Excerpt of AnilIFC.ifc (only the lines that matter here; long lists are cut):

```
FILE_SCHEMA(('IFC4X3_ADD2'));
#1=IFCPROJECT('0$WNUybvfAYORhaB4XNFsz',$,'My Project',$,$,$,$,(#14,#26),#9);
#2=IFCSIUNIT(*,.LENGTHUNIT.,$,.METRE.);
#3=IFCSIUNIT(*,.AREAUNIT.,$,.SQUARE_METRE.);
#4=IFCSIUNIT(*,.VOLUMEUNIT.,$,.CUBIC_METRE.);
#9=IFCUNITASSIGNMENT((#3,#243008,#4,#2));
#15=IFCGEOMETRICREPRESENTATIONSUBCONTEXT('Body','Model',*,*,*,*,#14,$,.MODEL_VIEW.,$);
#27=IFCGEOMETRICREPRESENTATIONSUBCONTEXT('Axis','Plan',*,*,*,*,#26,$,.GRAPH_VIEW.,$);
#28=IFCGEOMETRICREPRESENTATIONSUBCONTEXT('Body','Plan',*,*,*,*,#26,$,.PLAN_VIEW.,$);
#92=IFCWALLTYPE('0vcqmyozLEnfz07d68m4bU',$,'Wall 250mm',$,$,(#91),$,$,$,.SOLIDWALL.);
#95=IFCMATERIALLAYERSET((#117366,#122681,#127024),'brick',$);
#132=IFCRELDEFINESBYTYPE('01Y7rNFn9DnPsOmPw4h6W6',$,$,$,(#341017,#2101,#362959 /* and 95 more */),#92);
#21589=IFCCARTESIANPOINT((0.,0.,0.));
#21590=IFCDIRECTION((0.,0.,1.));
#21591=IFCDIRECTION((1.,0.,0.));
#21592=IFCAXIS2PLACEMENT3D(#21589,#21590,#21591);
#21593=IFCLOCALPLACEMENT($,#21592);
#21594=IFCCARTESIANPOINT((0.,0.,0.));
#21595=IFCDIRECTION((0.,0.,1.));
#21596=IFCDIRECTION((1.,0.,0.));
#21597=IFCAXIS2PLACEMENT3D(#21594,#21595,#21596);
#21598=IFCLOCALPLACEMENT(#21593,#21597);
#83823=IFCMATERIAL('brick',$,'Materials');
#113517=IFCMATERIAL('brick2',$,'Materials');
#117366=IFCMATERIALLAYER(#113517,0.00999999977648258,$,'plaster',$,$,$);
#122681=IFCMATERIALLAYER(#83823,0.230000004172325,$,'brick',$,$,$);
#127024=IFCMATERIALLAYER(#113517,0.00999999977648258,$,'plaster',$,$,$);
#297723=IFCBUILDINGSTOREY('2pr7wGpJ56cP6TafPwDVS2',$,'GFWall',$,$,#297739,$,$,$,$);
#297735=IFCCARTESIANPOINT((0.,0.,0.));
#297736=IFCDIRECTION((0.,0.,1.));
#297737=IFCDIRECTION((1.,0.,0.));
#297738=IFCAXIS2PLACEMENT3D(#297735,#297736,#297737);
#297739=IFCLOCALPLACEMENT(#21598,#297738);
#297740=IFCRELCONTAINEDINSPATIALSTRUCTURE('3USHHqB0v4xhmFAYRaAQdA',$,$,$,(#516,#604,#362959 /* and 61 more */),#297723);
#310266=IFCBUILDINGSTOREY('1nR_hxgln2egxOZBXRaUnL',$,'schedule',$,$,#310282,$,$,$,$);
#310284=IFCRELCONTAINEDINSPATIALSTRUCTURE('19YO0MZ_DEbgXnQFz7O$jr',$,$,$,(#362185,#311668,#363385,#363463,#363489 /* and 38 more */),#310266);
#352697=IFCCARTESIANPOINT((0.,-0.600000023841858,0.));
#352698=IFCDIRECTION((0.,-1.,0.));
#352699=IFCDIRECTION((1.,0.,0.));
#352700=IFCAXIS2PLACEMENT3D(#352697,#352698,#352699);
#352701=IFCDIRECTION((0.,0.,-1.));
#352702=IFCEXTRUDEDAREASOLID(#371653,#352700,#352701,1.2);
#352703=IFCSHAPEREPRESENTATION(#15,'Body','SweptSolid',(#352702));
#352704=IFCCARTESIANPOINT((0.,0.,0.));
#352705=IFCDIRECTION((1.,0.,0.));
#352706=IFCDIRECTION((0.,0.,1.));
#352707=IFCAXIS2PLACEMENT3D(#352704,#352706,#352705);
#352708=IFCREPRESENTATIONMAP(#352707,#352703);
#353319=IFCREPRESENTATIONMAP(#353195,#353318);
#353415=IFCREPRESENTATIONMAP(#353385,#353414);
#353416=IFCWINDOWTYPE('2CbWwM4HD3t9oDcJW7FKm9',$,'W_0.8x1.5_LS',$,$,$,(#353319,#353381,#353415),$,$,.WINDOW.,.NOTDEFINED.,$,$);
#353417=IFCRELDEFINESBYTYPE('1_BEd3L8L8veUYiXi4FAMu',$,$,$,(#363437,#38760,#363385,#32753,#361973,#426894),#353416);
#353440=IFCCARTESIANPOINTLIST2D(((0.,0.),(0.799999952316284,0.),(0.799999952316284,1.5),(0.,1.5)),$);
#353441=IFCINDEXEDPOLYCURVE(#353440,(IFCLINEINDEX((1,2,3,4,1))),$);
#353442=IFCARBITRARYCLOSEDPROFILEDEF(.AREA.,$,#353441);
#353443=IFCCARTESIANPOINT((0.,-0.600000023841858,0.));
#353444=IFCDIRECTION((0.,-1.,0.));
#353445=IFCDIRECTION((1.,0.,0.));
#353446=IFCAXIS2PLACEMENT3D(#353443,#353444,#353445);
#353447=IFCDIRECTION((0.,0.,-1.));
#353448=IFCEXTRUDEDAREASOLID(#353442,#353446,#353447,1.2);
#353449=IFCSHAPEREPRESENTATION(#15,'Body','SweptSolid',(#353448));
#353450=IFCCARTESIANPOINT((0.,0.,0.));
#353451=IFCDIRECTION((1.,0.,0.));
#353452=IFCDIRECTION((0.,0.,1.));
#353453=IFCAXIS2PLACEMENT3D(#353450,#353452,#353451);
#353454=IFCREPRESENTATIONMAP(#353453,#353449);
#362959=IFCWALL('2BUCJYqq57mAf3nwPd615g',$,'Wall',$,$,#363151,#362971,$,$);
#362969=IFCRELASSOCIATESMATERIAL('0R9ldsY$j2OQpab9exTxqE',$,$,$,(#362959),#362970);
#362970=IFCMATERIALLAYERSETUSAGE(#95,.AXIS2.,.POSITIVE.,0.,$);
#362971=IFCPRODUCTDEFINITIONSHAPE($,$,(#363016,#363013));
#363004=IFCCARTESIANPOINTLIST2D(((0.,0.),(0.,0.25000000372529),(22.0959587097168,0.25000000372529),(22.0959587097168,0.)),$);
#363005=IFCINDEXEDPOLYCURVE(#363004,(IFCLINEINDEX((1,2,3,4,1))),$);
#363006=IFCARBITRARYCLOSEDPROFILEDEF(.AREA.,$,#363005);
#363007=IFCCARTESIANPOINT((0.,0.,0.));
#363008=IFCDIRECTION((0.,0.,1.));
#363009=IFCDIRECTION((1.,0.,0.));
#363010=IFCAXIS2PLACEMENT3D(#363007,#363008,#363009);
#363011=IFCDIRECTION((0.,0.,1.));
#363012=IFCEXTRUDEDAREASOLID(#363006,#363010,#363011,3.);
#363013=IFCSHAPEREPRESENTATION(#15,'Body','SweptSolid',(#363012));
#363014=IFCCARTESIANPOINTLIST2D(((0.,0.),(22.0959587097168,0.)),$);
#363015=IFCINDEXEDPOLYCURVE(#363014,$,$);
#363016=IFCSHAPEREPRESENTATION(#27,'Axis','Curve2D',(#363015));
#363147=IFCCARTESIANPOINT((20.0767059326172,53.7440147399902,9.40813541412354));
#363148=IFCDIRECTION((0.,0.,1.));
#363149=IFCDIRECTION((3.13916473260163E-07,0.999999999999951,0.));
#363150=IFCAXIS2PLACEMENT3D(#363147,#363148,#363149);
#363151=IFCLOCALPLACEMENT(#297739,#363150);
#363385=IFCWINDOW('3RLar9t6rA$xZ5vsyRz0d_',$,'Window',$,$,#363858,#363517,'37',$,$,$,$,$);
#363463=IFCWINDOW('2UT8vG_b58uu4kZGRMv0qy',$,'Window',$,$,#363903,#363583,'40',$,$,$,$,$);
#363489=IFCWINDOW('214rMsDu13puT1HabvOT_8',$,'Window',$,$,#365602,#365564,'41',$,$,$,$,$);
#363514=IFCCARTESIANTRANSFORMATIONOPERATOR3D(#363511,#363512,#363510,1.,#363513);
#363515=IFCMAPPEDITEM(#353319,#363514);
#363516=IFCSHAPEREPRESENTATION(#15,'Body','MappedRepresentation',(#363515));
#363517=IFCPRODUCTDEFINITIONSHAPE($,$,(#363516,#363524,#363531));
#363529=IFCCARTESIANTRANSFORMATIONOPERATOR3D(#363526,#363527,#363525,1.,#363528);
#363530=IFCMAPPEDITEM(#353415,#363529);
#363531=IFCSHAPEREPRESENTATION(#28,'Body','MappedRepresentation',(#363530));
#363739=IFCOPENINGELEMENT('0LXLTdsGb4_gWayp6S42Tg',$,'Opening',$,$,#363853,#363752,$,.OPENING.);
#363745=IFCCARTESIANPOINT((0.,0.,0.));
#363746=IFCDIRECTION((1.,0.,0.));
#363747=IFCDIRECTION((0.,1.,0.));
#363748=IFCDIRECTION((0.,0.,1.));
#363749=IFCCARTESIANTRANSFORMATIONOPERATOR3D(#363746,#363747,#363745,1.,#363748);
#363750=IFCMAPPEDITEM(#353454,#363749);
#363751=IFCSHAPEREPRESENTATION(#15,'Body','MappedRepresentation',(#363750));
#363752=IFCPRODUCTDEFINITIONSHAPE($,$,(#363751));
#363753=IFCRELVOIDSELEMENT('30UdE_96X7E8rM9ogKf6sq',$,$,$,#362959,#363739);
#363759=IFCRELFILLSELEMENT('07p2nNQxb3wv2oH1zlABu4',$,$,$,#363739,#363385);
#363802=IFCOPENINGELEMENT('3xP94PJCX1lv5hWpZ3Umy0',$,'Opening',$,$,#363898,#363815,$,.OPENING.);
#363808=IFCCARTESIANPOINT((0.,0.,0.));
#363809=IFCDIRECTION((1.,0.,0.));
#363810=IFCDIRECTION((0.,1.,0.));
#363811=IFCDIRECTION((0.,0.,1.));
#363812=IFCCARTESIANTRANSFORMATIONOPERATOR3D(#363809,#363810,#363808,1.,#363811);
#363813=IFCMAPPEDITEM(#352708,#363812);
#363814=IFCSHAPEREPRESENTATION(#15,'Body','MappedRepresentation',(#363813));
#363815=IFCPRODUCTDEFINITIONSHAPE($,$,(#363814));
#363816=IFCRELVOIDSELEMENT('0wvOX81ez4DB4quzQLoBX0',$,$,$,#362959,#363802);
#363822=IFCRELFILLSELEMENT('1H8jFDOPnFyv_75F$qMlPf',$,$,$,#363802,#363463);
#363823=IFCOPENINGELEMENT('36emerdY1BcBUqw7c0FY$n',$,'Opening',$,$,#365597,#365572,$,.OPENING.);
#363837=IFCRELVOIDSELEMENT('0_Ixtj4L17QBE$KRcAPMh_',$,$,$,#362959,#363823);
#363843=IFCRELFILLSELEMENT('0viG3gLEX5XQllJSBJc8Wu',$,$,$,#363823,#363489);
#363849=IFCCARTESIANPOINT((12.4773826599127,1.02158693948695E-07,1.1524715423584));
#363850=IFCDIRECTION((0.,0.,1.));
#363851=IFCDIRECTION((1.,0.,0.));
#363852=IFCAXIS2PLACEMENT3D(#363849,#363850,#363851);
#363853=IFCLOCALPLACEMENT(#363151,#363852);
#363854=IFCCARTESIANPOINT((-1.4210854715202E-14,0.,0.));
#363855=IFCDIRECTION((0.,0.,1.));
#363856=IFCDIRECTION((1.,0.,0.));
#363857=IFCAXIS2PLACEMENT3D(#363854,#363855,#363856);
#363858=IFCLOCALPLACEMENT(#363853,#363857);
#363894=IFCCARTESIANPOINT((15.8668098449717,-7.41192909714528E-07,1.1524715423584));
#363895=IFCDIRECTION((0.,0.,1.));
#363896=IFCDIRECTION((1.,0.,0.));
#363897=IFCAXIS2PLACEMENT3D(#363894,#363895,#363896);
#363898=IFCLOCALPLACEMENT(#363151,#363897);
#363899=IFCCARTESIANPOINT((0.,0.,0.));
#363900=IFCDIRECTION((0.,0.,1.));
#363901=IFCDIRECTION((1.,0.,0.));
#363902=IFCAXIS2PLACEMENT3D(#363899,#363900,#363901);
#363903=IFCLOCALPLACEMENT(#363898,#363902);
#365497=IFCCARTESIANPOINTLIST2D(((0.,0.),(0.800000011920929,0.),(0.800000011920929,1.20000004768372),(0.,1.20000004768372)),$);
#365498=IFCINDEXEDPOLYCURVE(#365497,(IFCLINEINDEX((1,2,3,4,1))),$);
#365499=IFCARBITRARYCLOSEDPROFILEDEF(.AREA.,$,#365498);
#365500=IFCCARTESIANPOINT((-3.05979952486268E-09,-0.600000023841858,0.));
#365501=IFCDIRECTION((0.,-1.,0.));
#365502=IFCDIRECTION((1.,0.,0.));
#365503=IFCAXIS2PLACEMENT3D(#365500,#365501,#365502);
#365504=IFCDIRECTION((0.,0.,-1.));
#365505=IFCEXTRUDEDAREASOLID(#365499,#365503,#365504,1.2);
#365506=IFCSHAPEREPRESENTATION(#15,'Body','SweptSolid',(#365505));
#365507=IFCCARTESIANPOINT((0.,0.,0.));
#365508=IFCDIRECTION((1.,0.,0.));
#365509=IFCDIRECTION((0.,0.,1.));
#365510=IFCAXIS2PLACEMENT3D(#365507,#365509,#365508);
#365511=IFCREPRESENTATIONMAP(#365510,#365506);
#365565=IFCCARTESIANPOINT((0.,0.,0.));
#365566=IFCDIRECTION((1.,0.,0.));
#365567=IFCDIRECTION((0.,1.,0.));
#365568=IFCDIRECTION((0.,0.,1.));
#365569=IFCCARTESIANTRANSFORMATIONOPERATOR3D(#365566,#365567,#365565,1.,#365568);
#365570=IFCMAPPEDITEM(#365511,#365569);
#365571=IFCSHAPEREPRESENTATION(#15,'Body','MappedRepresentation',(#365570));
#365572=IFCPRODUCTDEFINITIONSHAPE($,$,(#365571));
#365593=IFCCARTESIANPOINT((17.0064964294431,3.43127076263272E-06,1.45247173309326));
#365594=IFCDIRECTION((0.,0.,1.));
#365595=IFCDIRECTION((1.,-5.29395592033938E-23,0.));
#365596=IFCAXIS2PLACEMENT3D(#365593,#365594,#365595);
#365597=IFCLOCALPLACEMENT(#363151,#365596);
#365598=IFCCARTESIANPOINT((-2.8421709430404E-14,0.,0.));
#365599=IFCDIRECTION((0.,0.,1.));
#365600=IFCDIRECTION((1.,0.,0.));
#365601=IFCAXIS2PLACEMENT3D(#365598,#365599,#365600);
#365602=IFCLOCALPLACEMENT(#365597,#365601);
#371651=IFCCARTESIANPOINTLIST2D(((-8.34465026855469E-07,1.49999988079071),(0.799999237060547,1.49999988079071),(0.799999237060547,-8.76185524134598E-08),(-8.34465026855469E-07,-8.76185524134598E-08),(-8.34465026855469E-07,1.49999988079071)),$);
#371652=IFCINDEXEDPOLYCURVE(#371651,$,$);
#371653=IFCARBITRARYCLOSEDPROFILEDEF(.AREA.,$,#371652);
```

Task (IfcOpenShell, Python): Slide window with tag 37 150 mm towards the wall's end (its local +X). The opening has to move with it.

```python
import ifcopenshell
import ifcopenshell.api.geometry
import ifcopenshell.util.placement
import ifcopenshell.util.unit

model = ifcopenshell.open("AnilIFC.ifc")
unit_scale = ifcopenshell.util.unit.calculate_unit_scale(model)

window = model.by_guid("3RLar9t6rA$xZ5vsyRz0d_")
opening = window.FillsVoids[0].RelatingOpeningElement
wall = opening.VoidsElements[0].RelatingBuildingElement

wall_matrix = ifcopenshell.util.placement.get_local_placement(wall.ObjectPlacement)
shift = wall_matrix[:3, 0] * 0.15 / unit_scale
before = ifcopenshell.util.placement.get_local_placement(window.ObjectPlacement)[:3, 3].copy()

# The window is placed relative to its opening, so it follows when the opening moves.
matrix = ifcopenshell.util.placement.get_local_placement(opening.ObjectPlacement)
matrix[:3, 3] += shift
ifcopenshell.api.geometry.edit_object_placement(
    model, product=opening, matrix=matrix, is_si=False, should_transform_children=True
)

after = ifcopenshell.util.placement.get_local_placement(window.ObjectPlacement)[:3, 3]
print("window moved by", (after - before).round(3) + 0.0)

model.write("AnilIFC_updated.ifc")
```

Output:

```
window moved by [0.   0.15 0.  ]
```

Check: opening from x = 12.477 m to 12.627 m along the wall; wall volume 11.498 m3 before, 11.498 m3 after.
